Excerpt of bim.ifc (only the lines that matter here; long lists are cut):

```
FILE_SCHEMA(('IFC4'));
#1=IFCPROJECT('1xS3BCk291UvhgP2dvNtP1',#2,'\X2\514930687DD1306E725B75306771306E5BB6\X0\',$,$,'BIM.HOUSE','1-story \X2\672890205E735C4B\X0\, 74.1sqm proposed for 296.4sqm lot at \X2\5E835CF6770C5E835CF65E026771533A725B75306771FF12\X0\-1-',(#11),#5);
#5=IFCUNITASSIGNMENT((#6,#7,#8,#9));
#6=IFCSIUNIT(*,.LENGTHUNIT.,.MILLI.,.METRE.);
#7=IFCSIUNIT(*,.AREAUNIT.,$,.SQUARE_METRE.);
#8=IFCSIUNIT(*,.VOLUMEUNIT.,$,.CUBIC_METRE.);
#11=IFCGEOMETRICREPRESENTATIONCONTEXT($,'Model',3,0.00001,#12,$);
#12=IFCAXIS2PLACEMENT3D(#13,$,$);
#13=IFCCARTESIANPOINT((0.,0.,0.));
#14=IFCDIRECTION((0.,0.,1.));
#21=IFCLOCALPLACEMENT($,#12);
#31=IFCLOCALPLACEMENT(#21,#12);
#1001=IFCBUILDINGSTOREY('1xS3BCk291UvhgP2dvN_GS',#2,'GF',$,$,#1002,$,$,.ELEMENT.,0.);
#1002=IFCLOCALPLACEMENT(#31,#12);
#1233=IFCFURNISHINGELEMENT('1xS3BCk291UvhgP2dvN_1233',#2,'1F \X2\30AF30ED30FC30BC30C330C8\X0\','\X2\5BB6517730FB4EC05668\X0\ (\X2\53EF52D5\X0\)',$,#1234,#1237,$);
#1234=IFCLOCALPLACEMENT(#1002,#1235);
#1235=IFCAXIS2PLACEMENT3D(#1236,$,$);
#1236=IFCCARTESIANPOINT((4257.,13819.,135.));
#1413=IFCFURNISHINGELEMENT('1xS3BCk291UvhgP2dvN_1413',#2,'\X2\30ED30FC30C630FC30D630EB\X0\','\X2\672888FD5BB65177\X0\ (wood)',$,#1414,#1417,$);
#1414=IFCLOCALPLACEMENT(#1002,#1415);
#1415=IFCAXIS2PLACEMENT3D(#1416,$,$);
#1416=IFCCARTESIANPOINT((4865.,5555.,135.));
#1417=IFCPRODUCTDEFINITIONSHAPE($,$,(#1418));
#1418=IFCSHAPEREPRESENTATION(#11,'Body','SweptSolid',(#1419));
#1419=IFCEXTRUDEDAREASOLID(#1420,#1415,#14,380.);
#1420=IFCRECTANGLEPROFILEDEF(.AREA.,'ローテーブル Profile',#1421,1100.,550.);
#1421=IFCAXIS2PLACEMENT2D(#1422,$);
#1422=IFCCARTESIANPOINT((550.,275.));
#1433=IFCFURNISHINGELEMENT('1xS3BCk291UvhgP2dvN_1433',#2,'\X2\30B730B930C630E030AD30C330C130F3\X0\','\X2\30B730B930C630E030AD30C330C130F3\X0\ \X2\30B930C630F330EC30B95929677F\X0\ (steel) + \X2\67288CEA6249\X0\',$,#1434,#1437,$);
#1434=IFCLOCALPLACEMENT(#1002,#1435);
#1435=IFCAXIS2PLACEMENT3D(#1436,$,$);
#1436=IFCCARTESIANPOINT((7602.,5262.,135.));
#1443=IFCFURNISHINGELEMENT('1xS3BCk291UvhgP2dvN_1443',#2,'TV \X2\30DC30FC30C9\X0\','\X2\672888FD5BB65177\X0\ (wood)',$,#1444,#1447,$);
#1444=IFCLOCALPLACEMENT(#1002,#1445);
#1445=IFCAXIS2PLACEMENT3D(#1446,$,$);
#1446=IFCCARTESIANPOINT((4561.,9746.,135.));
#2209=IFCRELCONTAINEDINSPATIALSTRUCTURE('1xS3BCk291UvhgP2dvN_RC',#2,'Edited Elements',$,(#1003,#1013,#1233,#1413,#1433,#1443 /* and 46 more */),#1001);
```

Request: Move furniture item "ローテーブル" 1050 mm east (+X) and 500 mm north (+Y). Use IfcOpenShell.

```python
import ifcopenshell
import ifcopenshell.api.geometry
import ifcopenshell.util.placement
import ifcopenshell.util.unit

model = ifcopenshell.open("bim.ifc")
unit_scale = ifcopenshell.util.unit.calculate_unit_scale(model)

item = model.by_guid("1xS3BCk291UvhgP2dvN_1413")
matrix = ifcopenshell.util.placement.get_local_placement(item.ObjectPlacement)
matrix[0, 3] += 1.05 / unit_scale
matrix[1, 3] += 0.5 / unit_scale
ifcopenshell.api.geometry.edit_object_placement(model, product=item, matrix=matrix, is_si=False)

print(ifcopenshell.util.placement.get_local_placement(item.ObjectPlacement).round(3) + 0.0)

model.write("bim_rev.ifc")
```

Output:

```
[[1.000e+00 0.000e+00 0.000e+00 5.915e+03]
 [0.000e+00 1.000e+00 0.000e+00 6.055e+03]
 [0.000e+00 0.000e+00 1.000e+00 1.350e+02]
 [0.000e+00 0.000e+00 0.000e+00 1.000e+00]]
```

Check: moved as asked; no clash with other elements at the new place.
